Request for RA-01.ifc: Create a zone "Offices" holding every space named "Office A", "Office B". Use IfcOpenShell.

First a look at what the model holds.

```python
import ifcopenshell

model = ifcopenshell.open("RA-01.ifc")
print(model.schema)
seen = {}
for space in model.by_type("IfcSpace"):
    seen[space.LongName] = seen.get(space.LongName, 0) + 1
for name, count in sorted(seen.items(), key=str):
    print(count, "x", name)
print("zones:", [z.Name for z in model.by_type("IfcZone")][:20])
```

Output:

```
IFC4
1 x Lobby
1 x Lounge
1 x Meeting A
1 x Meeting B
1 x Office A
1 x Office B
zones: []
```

```python
import ifcopenshell
import ifcopenshell.api.group
import ifcopenshell.api.root

model = ifcopenshell.open("RA-01.ifc")

names = {"Office A", "Office B"}
spaces = [s for s in model.by_type("IfcSpace") if s.LongName in names]

zone = ifcopenshell.api.root.create_entity(model, ifc_class="IfcZone", name="Offices")
ifcopenshell.api.group.assign_group(model, products=spaces, group=zone)
print(len(spaces), "spaces in", zone.Name)

model.write("RA-01_updated.ifc")
```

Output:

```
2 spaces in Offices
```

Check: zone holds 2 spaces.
